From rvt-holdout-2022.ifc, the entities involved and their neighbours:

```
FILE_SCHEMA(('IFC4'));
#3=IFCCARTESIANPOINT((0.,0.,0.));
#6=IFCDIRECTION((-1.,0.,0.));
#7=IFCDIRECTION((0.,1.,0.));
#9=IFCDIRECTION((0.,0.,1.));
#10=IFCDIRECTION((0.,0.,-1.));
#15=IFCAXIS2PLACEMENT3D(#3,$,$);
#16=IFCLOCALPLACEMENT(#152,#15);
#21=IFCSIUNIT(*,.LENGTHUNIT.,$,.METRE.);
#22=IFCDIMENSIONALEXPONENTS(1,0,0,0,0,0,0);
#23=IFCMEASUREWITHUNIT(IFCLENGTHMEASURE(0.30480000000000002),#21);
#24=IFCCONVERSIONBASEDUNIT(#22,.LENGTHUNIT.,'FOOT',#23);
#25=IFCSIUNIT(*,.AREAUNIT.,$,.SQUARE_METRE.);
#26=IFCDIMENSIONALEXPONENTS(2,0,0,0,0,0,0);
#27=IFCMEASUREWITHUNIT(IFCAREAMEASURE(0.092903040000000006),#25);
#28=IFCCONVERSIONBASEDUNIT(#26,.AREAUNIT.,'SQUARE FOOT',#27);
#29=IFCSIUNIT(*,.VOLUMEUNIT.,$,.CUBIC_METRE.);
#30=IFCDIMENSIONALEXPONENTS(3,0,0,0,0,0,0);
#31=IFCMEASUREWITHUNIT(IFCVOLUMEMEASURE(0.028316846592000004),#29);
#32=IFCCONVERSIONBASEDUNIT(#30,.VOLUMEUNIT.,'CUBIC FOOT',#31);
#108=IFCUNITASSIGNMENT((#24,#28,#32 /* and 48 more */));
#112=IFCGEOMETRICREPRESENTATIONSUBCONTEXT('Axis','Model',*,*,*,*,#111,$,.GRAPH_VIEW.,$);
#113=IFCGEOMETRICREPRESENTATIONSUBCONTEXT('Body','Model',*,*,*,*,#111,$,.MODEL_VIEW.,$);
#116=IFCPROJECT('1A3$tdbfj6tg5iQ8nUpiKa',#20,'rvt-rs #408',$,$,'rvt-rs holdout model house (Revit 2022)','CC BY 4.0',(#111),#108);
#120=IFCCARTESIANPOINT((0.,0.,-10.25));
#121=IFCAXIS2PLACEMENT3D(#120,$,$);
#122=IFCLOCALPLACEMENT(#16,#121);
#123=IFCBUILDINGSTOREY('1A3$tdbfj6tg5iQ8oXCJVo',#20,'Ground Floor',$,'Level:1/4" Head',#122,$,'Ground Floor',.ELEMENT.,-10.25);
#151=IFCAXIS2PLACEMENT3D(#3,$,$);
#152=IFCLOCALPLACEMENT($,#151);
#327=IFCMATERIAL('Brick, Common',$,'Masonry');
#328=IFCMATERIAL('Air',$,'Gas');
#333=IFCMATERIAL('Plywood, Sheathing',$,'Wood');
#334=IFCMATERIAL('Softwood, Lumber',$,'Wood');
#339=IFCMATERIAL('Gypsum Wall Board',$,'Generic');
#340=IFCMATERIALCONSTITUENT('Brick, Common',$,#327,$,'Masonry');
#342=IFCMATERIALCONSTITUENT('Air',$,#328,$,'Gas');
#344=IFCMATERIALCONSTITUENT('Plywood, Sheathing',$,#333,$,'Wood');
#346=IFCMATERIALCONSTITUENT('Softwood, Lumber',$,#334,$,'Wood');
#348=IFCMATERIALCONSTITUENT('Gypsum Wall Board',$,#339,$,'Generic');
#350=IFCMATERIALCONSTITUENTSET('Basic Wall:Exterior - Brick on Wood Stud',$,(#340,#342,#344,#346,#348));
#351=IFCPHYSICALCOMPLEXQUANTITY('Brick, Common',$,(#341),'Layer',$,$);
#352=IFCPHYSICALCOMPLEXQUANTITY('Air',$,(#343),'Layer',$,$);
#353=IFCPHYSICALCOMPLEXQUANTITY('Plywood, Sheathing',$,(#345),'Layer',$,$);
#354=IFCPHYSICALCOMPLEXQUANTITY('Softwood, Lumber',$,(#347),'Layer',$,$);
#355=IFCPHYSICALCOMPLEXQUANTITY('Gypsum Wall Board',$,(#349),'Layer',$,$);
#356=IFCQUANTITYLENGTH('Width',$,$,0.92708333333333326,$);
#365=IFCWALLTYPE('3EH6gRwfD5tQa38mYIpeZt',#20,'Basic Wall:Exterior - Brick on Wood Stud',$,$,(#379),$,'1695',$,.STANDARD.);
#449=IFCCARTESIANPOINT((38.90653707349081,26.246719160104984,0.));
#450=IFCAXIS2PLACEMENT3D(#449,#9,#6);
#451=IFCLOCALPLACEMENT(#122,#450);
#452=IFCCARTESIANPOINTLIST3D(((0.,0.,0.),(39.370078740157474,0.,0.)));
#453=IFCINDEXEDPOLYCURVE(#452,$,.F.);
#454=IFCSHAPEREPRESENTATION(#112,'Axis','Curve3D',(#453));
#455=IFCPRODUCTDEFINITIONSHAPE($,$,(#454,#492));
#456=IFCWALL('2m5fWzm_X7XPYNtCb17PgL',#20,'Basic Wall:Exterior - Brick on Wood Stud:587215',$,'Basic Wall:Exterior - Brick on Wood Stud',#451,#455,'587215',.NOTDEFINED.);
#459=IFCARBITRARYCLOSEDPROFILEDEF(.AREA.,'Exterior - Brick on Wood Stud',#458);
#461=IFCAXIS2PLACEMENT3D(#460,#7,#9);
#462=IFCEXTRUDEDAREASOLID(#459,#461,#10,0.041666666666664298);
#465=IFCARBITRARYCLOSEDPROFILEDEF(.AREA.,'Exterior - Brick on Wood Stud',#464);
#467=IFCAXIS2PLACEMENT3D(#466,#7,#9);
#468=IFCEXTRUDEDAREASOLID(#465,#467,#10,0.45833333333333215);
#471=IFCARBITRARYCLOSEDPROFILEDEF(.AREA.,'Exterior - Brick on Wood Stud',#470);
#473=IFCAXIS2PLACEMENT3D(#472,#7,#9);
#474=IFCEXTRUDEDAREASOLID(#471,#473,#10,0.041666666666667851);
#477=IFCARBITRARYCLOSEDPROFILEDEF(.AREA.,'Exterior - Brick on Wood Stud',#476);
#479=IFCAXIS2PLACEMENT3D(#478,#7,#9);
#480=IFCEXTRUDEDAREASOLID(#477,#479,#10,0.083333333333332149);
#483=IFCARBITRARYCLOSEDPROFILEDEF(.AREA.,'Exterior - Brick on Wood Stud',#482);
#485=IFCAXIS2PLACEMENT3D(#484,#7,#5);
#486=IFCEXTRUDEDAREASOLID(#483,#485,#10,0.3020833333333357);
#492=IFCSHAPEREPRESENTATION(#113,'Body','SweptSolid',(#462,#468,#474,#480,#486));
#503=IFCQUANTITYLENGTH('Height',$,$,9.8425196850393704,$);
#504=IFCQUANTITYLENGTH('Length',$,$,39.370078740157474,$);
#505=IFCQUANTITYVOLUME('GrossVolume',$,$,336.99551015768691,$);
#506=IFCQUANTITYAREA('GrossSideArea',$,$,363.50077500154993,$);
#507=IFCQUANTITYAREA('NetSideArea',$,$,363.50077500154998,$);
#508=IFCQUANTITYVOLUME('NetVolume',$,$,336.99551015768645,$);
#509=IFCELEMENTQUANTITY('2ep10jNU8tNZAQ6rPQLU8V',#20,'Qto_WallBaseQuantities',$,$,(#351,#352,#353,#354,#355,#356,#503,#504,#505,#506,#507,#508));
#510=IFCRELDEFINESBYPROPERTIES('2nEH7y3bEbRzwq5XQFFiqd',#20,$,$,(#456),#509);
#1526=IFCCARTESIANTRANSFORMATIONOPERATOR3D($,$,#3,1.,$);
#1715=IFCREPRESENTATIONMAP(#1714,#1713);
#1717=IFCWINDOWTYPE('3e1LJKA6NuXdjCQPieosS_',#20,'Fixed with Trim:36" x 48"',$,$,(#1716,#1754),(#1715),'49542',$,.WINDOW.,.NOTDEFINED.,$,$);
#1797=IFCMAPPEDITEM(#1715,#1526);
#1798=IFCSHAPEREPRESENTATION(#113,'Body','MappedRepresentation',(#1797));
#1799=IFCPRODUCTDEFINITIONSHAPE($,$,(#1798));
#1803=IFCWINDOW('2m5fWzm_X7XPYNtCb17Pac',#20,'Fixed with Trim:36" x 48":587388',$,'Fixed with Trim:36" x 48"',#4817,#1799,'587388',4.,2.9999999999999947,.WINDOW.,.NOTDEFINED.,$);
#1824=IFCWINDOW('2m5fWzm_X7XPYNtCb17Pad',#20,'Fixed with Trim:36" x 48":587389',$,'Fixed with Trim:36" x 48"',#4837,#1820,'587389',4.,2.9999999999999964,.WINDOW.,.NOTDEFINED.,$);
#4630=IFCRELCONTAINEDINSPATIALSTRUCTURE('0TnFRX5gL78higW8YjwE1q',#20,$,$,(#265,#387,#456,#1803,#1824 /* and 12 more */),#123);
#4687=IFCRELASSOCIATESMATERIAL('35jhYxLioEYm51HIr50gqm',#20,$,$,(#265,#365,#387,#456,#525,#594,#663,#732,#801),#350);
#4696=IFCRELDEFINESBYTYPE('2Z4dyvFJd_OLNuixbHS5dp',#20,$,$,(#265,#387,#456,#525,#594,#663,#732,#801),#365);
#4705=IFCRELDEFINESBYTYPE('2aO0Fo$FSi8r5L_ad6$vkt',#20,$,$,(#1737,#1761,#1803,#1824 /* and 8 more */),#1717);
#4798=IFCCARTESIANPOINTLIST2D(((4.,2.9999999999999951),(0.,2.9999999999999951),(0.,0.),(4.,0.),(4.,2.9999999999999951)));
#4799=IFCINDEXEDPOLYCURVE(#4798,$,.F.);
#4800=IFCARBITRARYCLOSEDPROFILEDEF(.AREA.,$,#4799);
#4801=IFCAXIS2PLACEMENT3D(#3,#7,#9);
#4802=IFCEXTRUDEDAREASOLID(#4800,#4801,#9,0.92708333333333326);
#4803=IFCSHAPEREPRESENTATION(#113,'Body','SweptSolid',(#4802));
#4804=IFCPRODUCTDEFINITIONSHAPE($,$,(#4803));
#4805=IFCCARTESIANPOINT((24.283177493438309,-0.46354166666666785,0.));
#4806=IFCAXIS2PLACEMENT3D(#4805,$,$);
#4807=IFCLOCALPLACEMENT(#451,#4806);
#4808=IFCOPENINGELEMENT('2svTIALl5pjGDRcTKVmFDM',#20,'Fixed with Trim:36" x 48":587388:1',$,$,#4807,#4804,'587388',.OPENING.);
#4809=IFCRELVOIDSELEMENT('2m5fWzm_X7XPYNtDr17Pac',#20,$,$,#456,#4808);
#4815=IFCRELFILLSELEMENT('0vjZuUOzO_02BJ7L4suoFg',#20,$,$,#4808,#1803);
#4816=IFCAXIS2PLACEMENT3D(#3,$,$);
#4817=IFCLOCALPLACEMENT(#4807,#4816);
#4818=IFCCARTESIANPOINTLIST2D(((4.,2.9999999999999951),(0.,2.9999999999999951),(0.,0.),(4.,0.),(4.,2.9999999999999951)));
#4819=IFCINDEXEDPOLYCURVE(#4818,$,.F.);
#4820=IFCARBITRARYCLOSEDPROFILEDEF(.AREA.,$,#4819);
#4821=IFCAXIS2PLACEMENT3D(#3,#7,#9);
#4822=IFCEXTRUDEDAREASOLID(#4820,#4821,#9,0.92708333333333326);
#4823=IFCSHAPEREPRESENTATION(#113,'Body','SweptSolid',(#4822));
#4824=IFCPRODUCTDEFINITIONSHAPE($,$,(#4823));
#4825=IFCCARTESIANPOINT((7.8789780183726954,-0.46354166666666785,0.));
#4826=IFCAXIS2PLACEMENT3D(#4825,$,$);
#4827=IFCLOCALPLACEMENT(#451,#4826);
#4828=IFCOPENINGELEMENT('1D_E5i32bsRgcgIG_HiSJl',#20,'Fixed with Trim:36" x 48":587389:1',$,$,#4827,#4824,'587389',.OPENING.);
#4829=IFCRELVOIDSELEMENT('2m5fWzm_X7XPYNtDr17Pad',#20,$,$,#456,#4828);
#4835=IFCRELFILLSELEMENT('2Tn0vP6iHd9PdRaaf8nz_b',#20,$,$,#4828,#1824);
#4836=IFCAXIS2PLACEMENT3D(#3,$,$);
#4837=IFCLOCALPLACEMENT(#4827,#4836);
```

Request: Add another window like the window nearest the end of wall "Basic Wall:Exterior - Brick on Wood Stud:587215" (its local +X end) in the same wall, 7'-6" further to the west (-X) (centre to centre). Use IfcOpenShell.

```python
import ifcopenshell
import ifcopenshell.api.feature
import ifcopenshell.api.geometry
import ifcopenshell.api.pset
import ifcopenshell.api.root
import ifcopenshell.geom
import ifcopenshell.util.element
import ifcopenshell.util.placement
import ifcopenshell.util.shape
import ifcopenshell.util.unit

model = ifcopenshell.open("rvt-holdout-2022.ifc")
unit_scale = ifcopenshell.util.unit.calculate_unit_scale(model)
area_scale = ifcopenshell.util.unit.calculate_unit_scale(model, "AREAUNIT")
volume_scale = ifcopenshell.util.unit.calculate_unit_scale(model, "VOLUMEUNIT")
settings = ifcopenshell.geom.settings()


def volume(element):
    """Net volume in cubic metres, openings subtracted."""
    shape = ifcopenshell.geom.create_shape(settings, element)
    return ifcopenshell.util.shape.get_volume(shape.geometry)


def reuse_history(source, copy):
    """copy_class also copies each property set's owner history, people and application; keep the originals."""
    for rel in copy.IsDefinedBy:
        if rel.is_a("IfcRelDefinesByProperties") and (history := rel.RelatingPropertyDefinition.OwnerHistory):
            rel.RelatingPropertyDefinition.OwnerHistory = source.OwnerHistory
            ifcopenshell.util.element.remove_deep2(model, history)


window = model.by_id(1803)
opening = window.FillsVoids[0].RelatingOpeningElement
wall = opening.VoidsElements[0].RelatingBuildingElement
before = volume(wall)
shift = ifcopenshell.util.placement.get_local_placement(wall.ObjectPlacement)[:3, 0] * 90 * 0.0254 / unit_scale

# copy_class copies the void relationship, type, container and properties, but no geometry.
new_opening = ifcopenshell.api.root.copy_class(model, product=opening)
new_opening.Representation = ifcopenshell.util.element.copy_deep(
    model, opening.Representation, exclude=["IfcGeometricRepresentationContext", "IfcRepresentationMap"]
)
new_opening.Name = 'Fixed with Trim:36" x 48"'
new_opening.Tag = None
reuse_history(opening, new_opening)
new_window = ifcopenshell.api.root.copy_class(model, product=window)
new_window.Representation = ifcopenshell.util.element.copy_deep(
    model, window.Representation, exclude=["IfcGeometricRepresentationContext", "IfcRepresentationMap"]
)
new_window.Name = 'Fixed with Trim:36" x 48"'
new_window.Tag = None
reuse_history(window, new_window)
ifcopenshell.api.feature.add_filling(model, opening=new_opening, element=new_window)

for old, new in ((opening, new_opening), (window, new_window)):
    matrix = ifcopenshell.util.placement.get_local_placement(old.ObjectPlacement)
    matrix[:3, 3] += shift
    ifcopenshell.api.geometry.edit_object_placement(model, product=new, matrix=matrix, is_si=False)

after = volume(wall)
thickness = 0.2826  # wall thickness in metres

# Update the wall's stored quantities.
qto = model.by_id(ifcopenshell.util.element.get_pset(wall, "Qto_WallBaseQuantities", should_inherit=False)["id"])
ifcopenshell.api.pset.edit_qto(model, qto=qto, properties={
    "NetSideArea": after / thickness / area_scale,
    "NetVolume": after / volume_scale,
})

print(f"wall volume {before:.3f} -> {after:.3f} m3")

model.write("rvt-holdout-2022_rev.ifc")
```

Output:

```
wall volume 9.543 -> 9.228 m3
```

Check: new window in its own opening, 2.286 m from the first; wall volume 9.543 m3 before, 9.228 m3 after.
